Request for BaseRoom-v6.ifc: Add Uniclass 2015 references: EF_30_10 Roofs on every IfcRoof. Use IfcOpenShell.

First a look at what the model holds.

```python
import ifcopenshell

model = ifcopenshell.open("BaseRoom-v6.ifc")
print(model.schema)
print("classifications:", [c.Name for c in model.by_type("IfcClassification")])
for ifc_class in ("IfcDoor", "IfcRoof", "IfcStair", "IfcWall", "IfcWindow"):
    print(ifc_class, len(model.by_type(ifc_class)))
```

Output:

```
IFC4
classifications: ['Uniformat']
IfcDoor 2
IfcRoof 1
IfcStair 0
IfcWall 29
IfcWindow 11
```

```python
import ifcopenshell
import ifcopenshell.api.classification

model = ifcopenshell.open("BaseRoom-v6.ifc")

system = ifcopenshell.api.classification.add_classification(model, classification="Uniclass 2015")

codes = {
    "IfcRoof": ("EF_30_10", "Roofs"),
}
for ifc_class, (code, name) in codes.items():
    products = model.by_type(ifc_class)
    ifcopenshell.api.classification.add_reference(
        model, products=products, classification=system, identification=code, name=name
    )
    print(code, len(products))

model.write("BaseRoom-v6_rev.ifc")
```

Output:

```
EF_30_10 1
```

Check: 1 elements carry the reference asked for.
